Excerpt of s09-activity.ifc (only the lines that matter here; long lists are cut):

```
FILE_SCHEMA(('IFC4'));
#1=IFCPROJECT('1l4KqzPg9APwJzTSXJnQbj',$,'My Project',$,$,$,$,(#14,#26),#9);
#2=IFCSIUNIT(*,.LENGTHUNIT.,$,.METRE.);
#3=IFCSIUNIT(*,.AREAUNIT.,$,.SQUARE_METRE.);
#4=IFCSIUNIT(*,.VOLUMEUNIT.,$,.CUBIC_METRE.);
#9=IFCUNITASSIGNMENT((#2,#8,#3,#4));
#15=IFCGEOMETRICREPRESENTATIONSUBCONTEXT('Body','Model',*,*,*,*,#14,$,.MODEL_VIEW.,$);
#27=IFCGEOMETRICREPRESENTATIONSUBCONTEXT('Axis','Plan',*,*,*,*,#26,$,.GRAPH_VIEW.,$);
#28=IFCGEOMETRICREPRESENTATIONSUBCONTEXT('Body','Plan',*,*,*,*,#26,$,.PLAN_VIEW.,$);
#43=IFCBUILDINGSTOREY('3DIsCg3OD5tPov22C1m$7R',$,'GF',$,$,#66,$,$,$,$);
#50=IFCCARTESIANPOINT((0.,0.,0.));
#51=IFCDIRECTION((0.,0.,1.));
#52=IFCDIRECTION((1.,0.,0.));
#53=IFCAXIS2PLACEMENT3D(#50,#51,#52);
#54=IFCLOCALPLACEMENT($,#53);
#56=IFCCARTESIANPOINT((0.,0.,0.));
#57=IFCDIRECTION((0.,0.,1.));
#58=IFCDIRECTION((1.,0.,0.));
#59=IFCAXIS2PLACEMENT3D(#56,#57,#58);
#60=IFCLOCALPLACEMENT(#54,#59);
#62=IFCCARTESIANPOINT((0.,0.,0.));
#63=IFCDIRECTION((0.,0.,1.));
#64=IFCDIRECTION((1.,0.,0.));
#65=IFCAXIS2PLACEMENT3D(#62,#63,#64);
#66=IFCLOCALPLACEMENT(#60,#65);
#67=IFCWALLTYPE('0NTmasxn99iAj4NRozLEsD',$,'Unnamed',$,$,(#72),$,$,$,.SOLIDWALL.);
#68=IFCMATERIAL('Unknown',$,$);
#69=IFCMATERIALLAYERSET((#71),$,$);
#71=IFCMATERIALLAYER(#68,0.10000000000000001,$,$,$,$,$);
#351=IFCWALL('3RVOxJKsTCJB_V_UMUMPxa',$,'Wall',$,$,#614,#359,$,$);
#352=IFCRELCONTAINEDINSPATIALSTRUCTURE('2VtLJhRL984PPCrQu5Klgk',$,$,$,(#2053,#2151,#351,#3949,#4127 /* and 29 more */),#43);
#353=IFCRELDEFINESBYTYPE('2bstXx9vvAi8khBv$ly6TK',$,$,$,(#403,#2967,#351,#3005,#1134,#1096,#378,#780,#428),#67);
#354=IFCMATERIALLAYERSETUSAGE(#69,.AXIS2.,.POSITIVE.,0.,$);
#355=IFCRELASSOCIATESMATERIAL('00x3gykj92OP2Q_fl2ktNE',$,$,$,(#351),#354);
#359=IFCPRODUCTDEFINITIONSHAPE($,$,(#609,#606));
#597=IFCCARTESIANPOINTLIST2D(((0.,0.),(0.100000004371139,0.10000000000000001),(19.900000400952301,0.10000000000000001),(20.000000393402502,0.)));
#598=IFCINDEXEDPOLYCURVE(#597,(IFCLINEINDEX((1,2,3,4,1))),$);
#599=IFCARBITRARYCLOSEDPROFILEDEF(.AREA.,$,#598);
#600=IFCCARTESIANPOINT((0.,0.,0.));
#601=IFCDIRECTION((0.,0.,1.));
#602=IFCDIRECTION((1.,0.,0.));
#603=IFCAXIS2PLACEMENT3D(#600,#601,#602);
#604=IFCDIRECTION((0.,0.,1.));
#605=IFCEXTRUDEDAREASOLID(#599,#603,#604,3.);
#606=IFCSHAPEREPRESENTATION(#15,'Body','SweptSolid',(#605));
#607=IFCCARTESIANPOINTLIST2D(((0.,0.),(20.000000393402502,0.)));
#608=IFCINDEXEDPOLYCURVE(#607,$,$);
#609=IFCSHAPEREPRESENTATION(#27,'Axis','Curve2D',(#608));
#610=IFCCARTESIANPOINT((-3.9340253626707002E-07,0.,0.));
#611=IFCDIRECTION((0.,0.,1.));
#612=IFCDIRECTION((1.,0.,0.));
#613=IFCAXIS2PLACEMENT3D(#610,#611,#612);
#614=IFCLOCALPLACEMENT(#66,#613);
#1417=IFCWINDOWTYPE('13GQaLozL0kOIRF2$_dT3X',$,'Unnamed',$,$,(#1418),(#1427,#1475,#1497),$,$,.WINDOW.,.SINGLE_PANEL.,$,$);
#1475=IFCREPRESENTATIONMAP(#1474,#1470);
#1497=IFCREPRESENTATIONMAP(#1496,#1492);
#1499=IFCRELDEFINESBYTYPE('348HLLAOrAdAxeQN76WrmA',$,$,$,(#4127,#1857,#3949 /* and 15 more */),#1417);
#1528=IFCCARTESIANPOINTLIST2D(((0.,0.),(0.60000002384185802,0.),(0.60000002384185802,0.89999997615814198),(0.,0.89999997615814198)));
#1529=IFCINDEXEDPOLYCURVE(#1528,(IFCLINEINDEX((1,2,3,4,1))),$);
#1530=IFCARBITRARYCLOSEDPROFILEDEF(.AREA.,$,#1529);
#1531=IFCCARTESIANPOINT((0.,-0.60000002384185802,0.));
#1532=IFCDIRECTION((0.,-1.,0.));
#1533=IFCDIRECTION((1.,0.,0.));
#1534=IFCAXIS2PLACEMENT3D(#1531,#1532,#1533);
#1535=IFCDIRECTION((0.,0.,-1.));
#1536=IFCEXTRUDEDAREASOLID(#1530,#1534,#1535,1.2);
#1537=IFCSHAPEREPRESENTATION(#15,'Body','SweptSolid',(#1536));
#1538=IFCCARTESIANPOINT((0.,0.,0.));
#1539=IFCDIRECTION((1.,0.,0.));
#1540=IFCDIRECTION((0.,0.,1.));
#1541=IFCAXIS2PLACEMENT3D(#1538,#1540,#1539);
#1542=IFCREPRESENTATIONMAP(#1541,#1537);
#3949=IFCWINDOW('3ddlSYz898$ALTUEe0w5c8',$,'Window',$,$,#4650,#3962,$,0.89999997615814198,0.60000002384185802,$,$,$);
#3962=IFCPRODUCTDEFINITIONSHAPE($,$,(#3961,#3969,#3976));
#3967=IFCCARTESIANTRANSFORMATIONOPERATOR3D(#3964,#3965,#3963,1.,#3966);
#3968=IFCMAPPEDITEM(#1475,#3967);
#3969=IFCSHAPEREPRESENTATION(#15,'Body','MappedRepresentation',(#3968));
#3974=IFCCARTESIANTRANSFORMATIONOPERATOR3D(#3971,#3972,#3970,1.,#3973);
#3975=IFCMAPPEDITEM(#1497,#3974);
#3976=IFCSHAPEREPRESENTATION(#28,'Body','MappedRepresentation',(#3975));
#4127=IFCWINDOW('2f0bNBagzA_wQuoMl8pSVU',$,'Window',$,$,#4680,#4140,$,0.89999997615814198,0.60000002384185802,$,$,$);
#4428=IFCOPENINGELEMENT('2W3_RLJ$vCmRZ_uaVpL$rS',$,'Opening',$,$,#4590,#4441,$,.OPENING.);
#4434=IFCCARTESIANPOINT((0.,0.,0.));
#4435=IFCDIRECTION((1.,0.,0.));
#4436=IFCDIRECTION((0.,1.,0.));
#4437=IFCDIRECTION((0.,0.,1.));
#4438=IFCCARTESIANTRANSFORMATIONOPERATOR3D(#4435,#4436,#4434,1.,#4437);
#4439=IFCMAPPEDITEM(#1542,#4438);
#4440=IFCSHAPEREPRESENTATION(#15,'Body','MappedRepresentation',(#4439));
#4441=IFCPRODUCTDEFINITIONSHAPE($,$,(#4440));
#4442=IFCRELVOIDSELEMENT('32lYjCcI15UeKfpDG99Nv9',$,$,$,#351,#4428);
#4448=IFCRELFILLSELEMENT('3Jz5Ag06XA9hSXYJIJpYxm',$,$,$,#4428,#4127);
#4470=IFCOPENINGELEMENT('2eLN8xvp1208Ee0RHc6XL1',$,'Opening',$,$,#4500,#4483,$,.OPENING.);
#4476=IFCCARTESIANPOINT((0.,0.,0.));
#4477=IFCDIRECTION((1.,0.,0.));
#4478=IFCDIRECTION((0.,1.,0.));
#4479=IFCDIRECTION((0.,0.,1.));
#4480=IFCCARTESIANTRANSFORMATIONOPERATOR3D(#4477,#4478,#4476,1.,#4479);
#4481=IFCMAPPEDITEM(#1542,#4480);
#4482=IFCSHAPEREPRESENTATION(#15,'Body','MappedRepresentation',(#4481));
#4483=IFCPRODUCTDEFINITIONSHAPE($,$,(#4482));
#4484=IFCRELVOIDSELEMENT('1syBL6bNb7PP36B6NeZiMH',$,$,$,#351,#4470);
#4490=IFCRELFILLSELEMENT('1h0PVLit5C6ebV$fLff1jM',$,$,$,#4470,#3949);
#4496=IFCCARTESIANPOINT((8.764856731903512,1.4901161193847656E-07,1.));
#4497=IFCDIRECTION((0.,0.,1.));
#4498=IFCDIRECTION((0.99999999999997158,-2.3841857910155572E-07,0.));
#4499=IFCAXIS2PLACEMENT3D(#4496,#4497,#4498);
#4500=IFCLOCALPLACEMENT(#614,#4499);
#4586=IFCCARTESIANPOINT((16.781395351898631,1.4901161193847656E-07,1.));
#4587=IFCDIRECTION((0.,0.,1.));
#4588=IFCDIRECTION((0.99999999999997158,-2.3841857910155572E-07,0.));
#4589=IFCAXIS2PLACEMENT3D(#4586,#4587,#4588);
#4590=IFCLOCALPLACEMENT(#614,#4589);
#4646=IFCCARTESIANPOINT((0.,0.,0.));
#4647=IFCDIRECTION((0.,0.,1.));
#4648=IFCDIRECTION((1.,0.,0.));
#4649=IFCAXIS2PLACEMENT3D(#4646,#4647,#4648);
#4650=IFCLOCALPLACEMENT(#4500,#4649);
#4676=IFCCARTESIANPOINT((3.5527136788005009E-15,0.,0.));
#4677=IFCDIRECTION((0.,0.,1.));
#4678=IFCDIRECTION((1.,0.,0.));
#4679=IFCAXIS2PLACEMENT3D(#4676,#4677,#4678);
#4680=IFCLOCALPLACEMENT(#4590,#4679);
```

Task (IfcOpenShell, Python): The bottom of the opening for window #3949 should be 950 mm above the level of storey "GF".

```python
import numpy as np
import ifcopenshell
import ifcopenshell.api.geometry
import ifcopenshell.geom
import ifcopenshell.util.element
import ifcopenshell.util.placement
import ifcopenshell.util.shape
import ifcopenshell.util.unit

model = ifcopenshell.open("s09-activity.ifc")
unit_scale = ifcopenshell.util.unit.calculate_unit_scale(model)

window = model.by_guid("3ddlSYz898$ALTUEe0w5c8")
opening = window.FillsVoids[0].RelatingOpeningElement
storey = ifcopenshell.util.element.get_container(window, ifc_class="IfcBuildingStorey")
level = ifcopenshell.util.placement.get_local_placement(storey.ObjectPlacement)[2, 3]

# The opening's origin need not be at the sill, so measure its lowest point.
shape = ifcopenshell.geom.create_shape(ifcopenshell.geom.settings(), opening)
bottom = ifcopenshell.util.shape.get_shape_bottom_elevation(shape, shape.geometry) / unit_scale
dz = level + 0.95 / unit_scale - bottom

shift = np.array([0.0, 0.0, dz])
# The window is placed relative to its opening, so it follows when the opening moves.
matrix = ifcopenshell.util.placement.get_local_placement(opening.ObjectPlacement)
matrix[:3, 3] += shift
ifcopenshell.api.geometry.edit_object_placement(
    model, product=opening, matrix=matrix, is_si=False, should_transform_children=True
)

print(f"moved by {dz * unit_scale:+.3f} m")

model.write("s09-activity_rev.ifc")
```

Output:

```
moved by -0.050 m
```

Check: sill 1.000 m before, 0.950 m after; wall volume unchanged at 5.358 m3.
